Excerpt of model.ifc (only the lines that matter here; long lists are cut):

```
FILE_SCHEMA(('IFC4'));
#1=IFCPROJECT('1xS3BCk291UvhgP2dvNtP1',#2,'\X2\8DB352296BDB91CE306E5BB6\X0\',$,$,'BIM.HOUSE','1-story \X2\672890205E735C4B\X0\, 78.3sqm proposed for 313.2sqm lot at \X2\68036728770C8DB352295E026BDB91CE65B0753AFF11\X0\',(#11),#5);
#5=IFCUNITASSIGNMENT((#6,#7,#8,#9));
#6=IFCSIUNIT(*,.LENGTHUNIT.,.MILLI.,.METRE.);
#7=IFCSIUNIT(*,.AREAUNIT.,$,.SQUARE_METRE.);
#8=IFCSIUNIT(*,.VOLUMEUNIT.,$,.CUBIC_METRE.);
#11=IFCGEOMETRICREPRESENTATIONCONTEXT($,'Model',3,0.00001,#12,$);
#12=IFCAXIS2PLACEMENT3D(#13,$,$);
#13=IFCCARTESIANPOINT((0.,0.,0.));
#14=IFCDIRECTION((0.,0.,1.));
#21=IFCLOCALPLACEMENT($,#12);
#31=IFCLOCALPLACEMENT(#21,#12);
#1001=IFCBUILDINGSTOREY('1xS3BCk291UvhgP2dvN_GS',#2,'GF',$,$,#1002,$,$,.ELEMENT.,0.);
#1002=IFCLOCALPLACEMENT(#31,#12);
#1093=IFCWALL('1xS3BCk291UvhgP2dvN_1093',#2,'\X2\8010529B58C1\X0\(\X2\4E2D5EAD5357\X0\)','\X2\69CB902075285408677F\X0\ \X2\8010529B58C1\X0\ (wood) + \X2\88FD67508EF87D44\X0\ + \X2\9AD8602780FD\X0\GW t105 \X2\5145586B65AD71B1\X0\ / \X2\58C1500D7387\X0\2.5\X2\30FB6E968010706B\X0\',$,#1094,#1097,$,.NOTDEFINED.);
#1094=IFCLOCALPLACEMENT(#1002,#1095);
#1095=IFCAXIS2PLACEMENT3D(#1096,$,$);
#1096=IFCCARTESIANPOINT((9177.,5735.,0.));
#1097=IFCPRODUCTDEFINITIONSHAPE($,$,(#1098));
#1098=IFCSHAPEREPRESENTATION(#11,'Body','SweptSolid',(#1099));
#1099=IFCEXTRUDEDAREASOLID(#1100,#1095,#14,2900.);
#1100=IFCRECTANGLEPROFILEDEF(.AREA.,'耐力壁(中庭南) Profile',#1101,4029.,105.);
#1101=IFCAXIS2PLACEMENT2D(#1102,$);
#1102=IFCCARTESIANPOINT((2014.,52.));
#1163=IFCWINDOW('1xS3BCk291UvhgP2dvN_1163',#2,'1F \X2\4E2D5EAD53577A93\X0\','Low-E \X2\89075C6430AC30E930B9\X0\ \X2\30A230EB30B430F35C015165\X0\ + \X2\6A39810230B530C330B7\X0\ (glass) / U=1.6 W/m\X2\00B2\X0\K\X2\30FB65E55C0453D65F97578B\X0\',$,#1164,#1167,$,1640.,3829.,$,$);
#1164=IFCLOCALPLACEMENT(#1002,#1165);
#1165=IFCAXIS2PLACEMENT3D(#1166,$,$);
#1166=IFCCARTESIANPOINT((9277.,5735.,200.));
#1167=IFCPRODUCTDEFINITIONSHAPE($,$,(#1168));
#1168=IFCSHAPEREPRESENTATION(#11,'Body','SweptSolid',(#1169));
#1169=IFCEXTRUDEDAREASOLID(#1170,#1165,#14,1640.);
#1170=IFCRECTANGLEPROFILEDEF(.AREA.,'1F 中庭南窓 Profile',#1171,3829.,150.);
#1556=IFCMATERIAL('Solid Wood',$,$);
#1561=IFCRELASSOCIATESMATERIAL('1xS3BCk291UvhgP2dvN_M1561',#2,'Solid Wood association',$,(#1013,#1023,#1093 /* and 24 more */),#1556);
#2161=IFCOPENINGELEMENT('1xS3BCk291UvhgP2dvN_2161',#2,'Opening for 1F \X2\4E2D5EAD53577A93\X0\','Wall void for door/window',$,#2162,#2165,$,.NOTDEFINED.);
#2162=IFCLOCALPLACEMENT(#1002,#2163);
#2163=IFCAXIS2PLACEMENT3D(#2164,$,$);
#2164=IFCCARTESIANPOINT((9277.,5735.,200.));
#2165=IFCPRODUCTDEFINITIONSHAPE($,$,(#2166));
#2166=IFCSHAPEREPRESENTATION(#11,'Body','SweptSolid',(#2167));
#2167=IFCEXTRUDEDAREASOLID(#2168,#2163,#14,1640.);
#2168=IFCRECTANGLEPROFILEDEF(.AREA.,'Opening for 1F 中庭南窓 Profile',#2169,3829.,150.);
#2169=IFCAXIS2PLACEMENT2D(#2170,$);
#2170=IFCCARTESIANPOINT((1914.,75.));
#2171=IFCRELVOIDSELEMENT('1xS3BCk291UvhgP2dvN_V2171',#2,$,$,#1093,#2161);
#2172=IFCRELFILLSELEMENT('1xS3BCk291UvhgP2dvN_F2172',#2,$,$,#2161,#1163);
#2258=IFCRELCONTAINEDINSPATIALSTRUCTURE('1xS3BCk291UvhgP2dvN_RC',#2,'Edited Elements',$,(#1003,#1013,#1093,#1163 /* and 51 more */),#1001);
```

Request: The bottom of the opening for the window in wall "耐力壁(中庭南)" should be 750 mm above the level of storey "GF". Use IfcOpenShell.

```python
import numpy as np
import ifcopenshell
import ifcopenshell.api.geometry
import ifcopenshell.geom
import ifcopenshell.util.element
import ifcopenshell.util.placement
import ifcopenshell.util.shape
import ifcopenshell.util.unit

model = ifcopenshell.open("model.ifc")
unit_scale = ifcopenshell.util.unit.calculate_unit_scale(model)

window = model.by_guid("1xS3BCk291UvhgP2dvN_1163")
opening = window.FillsVoids[0].RelatingOpeningElement
storey = ifcopenshell.util.element.get_container(window, ifc_class="IfcBuildingStorey")
level = ifcopenshell.util.placement.get_local_placement(storey.ObjectPlacement)[2, 3]

# The opening's origin need not be at the sill, so measure its lowest point.
shape = ifcopenshell.geom.create_shape(ifcopenshell.geom.settings(), opening)
bottom = ifcopenshell.util.shape.get_shape_bottom_elevation(shape, shape.geometry) / unit_scale
dz = level + 0.75 / unit_scale - bottom

shift = np.array([0.0, 0.0, dz])
# The window is not placed relative to its opening, so move both.
for product in (opening, window):
    matrix = ifcopenshell.util.placement.get_local_placement(product.ObjectPlacement)
    matrix[:3, 3] += shift
    ifcopenshell.api.geometry.edit_object_placement(model, product=product, matrix=matrix, is_si=False)

print(f"moved by {dz * unit_scale:+.3f} m")

model.write("model_rev.ifc")
```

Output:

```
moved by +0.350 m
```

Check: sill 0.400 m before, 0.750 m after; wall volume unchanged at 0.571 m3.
